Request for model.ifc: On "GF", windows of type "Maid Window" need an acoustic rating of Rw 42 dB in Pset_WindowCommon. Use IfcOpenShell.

First a look at what the model holds.

```python
import ifcopenshell
import ifcopenshell.util.element

model = ifcopenshell.open("model.ifc")
print(model.schema)
storey = next(s for s in model.by_type("IfcBuildingStorey") if s.Name == "GF")
windows = [e for e in ifcopenshell.util.element.get_decomposition(storey) if e.is_a("IfcWindow")]
seen = {}
for e in windows:
    element_type = ifcopenshell.util.element.get_type(e)
    key = (element_type.Name if element_type != e and element_type else None, ifcopenshell.util.element.get_pset(e, "Pset_WindowCommon", "AcousticRating"))
    seen[key] = seen.get(key, 0) + 1
for (name, value), count in sorted(seen.items(), key=str):
    print(count, "x", name, "|", value)
```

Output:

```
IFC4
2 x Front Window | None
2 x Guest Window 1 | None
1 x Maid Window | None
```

```python
import ifcopenshell
import ifcopenshell.api.pset
import ifcopenshell.util.element

model = ifcopenshell.open("model.ifc")

storey = next(s for s in model.by_type("IfcBuildingStorey") if s.Name == "GF")
windows = [e for e in ifcopenshell.util.element.get_decomposition(storey) if e.is_a("IfcWindow")]

count = 0
for e in windows:
    element_type = ifcopenshell.util.element.get_type(e)
    if element_type in (None, e) or element_type.Name != "Maid Window":
        continue
    # add_pset returns the element's existing set when there is one.
    pset = ifcopenshell.api.pset.add_pset(model, product=e, name="Pset_WindowCommon")
    ifcopenshell.api.pset.edit_pset(model, pset=pset, properties={"AcousticRating": "Rw 42 dB"})
    count += 1

print(count, "windows updated")

model.write("model_rev.ifc")
```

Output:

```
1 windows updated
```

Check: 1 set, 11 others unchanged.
